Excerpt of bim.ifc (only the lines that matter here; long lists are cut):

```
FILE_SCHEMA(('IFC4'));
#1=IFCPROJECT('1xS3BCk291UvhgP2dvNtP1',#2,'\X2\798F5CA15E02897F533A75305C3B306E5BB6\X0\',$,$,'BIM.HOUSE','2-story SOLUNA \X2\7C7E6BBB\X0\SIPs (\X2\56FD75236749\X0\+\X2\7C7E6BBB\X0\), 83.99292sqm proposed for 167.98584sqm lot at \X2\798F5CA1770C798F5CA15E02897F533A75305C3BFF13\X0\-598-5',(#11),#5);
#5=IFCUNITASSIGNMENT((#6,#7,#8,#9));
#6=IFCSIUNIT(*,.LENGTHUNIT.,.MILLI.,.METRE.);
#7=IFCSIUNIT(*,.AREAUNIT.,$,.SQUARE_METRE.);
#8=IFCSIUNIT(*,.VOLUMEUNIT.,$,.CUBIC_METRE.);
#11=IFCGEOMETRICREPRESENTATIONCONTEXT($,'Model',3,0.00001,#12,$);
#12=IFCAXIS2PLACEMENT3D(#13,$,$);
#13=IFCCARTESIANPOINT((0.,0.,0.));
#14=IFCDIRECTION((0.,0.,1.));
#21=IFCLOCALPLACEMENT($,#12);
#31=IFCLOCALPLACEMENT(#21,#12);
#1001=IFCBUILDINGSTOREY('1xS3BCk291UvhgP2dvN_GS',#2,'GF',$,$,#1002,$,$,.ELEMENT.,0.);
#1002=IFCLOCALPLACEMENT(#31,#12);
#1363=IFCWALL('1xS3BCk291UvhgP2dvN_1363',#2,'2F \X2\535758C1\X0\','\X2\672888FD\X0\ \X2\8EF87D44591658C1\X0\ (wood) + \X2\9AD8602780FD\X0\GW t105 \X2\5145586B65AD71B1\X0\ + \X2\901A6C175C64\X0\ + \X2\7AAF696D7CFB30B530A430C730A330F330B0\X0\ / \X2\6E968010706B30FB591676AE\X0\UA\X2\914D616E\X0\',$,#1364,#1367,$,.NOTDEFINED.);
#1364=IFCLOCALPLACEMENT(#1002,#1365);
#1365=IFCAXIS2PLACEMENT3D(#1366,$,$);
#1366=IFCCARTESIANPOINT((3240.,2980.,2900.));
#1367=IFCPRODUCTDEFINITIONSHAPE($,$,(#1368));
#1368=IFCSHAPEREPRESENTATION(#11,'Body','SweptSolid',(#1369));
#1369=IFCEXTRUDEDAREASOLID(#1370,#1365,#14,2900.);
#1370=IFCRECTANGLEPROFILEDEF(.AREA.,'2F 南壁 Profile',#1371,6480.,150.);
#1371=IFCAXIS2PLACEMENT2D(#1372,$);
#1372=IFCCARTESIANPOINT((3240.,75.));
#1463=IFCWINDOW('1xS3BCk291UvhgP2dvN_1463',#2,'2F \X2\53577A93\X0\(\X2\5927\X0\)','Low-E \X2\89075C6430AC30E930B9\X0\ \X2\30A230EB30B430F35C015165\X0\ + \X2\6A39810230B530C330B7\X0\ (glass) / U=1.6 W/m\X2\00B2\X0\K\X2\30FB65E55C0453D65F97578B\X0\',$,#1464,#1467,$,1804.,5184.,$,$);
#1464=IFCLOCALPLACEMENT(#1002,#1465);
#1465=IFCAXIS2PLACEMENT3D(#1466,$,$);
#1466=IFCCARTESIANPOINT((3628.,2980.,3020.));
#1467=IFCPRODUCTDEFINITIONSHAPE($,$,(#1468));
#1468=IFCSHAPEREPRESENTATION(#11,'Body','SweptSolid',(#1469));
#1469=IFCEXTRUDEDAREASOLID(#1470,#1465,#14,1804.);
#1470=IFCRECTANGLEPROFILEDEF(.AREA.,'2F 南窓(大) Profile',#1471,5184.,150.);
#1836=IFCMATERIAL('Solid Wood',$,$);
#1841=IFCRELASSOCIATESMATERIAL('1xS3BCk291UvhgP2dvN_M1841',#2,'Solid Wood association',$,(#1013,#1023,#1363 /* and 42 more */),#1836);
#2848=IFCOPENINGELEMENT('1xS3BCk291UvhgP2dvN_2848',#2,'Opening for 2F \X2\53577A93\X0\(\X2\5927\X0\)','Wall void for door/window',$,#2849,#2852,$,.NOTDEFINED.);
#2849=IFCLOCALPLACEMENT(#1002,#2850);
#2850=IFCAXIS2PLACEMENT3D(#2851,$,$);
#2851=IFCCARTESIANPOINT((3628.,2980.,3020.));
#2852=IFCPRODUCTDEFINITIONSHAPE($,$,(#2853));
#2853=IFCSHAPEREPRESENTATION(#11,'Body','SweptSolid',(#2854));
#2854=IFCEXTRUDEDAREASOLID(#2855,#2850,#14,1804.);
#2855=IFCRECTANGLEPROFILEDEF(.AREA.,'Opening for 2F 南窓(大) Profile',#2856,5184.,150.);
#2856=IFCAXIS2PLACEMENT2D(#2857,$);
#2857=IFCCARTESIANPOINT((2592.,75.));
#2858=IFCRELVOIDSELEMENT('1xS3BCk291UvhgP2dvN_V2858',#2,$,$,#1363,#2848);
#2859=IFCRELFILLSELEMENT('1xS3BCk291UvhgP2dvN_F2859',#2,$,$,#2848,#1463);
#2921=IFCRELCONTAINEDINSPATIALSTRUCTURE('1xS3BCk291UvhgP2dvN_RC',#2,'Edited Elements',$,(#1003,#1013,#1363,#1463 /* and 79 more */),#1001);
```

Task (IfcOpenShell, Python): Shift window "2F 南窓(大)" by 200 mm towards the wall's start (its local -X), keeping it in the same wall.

```python
import ifcopenshell
import ifcopenshell.api.geometry
import ifcopenshell.util.placement

model = ifcopenshell.open("bim.ifc")

window = model.by_guid("1xS3BCk291UvhgP2dvN_1463")
opening = window.FillsVoids[0].RelatingOpeningElement
wall = opening.VoidsElements[0].RelatingBuildingElement

wall_matrix = ifcopenshell.util.placement.get_local_placement(wall.ObjectPlacement)
shift = wall_matrix[:3, 0] * -200.0
before = ifcopenshell.util.placement.get_local_placement(window.ObjectPlacement)[:3, 3].copy()

# The window is not placed relative to its opening, so move both.
for product in (opening, window):
    matrix = ifcopenshell.util.placement.get_local_placement(product.ObjectPlacement)
    matrix[:3, 3] += shift
    ifcopenshell.api.geometry.edit_object_placement(model, product=product, matrix=matrix, is_si=False)

after = ifcopenshell.util.placement.get_local_placement(window.ObjectPlacement)[:3, 3]
print("window moved by", (after - before).round(3) + 0.0)

model.write("bim_updated.ifc")
```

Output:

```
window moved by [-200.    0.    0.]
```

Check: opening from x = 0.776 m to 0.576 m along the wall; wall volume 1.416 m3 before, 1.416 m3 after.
